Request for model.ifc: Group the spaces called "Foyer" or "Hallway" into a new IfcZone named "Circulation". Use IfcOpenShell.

First a look at what the model holds.

```python
import ifcopenshell

model = ifcopenshell.open("model.ifc")
print(model.schema)
seen = {}
for space in model.by_type("IfcSpace"):
    seen[space.LongName] = seen.get(space.LongName, 0) + 1
for name, count in sorted(seen.items(), key=str):
    print(count, "x", name)
print("zones:", [z.Name for z in model.by_type("IfcZone")][:20])
```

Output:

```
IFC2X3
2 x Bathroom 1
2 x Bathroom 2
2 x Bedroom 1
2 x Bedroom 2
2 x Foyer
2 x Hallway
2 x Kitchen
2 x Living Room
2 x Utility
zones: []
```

```python
import ifcopenshell
import ifcopenshell.api.group
import ifcopenshell.api.root

model = ifcopenshell.open("model.ifc")

names = {"Foyer", "Hallway"}
spaces = [s for s in model.by_type("IfcSpace") if s.LongName in names]

zone = ifcopenshell.api.root.create_entity(model, ifc_class="IfcZone", name="Circulation")
ifcopenshell.api.group.assign_group(model, products=spaces, group=zone)
print(len(spaces), "spaces in", zone.Name)

model.write("model_updated.ifc")
```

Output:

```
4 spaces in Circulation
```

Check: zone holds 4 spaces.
